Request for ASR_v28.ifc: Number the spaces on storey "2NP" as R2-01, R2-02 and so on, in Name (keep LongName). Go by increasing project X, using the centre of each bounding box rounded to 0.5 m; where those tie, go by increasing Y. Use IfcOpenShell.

First a look at what the model holds.

```python
import ifcopenshell
import ifcopenshell.util.element
import ifcopenshell.util.placement

model = ifcopenshell.open("ASR_v28.ifc")
print(model.schema)
storey = next(s for s in model.by_type("IfcBuildingStorey") if s.Name == "2NP")
spaces = [e for e in ifcopenshell.util.element.get_decomposition(storey) if e.is_a("IfcSpace")]
for e in sorted(spaces, key=lambda e: e.id()):
    origin = ifcopenshell.util.placement.get_local_placement(e.ObjectPlacement)[:3, 3]
    print(e.id(), e.Name, e.LongName, origin.round(2) + 0.0, sep=" | ")
```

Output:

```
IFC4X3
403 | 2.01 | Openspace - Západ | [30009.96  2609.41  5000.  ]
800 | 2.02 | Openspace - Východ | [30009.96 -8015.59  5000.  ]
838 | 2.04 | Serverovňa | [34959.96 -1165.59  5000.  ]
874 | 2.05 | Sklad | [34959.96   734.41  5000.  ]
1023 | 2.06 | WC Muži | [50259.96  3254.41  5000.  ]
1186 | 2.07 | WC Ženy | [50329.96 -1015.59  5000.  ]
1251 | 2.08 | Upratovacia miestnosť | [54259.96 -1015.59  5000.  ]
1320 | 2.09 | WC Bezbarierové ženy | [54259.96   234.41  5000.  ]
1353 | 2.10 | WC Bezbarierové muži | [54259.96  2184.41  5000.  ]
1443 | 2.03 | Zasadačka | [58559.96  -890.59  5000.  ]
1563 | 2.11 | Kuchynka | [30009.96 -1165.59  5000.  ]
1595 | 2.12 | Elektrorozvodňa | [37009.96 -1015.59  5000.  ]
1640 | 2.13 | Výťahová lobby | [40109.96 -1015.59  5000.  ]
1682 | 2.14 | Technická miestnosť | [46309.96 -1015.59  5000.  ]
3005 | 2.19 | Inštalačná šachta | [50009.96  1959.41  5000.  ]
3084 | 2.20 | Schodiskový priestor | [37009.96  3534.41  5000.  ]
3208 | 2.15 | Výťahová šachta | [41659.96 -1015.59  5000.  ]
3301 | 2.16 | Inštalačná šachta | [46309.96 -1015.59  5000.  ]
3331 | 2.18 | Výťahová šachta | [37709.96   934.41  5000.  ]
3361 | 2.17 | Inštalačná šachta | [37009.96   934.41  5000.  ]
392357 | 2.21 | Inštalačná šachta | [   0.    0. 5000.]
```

```python
import ifcopenshell
import ifcopenshell.geom
import ifcopenshell.util.element
import ifcopenshell.util.shape

model = ifcopenshell.open("ASR_v28.ifc")
settings = ifcopenshell.geom.settings()
settings.set("use-world-coords", True)


def centre(element):
    shape = ifcopenshell.geom.create_shape(settings, element)
    return ifcopenshell.util.shape.get_bbox_centroid(shape.geometry)


storey = next(s for s in model.by_type("IfcBuildingStorey") if s.Name == "2NP")
spaces = [e for e in ifcopenshell.util.element.get_decomposition(storey) if e.is_a("IfcSpace")]

# Insertion points can sit at a corner or the storey origin, so sort by the geometry (in metres).
centres = {e: centre(e) for e in spaces}
spaces.sort(key=lambda e: (round(centres[e][0] / 0.5), centres[e][1]))

for i, e in enumerate(spaces, start=1):
    number = f"R2-{i:02d}"
    e.Name = number
    print(e.id(), number)

model.write("ASR_v28_v2.ifc")
```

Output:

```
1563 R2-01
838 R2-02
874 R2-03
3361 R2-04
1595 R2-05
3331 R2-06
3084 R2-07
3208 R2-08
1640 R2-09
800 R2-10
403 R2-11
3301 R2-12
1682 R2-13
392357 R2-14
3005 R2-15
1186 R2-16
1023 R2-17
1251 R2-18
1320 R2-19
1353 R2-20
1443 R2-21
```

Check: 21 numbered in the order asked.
